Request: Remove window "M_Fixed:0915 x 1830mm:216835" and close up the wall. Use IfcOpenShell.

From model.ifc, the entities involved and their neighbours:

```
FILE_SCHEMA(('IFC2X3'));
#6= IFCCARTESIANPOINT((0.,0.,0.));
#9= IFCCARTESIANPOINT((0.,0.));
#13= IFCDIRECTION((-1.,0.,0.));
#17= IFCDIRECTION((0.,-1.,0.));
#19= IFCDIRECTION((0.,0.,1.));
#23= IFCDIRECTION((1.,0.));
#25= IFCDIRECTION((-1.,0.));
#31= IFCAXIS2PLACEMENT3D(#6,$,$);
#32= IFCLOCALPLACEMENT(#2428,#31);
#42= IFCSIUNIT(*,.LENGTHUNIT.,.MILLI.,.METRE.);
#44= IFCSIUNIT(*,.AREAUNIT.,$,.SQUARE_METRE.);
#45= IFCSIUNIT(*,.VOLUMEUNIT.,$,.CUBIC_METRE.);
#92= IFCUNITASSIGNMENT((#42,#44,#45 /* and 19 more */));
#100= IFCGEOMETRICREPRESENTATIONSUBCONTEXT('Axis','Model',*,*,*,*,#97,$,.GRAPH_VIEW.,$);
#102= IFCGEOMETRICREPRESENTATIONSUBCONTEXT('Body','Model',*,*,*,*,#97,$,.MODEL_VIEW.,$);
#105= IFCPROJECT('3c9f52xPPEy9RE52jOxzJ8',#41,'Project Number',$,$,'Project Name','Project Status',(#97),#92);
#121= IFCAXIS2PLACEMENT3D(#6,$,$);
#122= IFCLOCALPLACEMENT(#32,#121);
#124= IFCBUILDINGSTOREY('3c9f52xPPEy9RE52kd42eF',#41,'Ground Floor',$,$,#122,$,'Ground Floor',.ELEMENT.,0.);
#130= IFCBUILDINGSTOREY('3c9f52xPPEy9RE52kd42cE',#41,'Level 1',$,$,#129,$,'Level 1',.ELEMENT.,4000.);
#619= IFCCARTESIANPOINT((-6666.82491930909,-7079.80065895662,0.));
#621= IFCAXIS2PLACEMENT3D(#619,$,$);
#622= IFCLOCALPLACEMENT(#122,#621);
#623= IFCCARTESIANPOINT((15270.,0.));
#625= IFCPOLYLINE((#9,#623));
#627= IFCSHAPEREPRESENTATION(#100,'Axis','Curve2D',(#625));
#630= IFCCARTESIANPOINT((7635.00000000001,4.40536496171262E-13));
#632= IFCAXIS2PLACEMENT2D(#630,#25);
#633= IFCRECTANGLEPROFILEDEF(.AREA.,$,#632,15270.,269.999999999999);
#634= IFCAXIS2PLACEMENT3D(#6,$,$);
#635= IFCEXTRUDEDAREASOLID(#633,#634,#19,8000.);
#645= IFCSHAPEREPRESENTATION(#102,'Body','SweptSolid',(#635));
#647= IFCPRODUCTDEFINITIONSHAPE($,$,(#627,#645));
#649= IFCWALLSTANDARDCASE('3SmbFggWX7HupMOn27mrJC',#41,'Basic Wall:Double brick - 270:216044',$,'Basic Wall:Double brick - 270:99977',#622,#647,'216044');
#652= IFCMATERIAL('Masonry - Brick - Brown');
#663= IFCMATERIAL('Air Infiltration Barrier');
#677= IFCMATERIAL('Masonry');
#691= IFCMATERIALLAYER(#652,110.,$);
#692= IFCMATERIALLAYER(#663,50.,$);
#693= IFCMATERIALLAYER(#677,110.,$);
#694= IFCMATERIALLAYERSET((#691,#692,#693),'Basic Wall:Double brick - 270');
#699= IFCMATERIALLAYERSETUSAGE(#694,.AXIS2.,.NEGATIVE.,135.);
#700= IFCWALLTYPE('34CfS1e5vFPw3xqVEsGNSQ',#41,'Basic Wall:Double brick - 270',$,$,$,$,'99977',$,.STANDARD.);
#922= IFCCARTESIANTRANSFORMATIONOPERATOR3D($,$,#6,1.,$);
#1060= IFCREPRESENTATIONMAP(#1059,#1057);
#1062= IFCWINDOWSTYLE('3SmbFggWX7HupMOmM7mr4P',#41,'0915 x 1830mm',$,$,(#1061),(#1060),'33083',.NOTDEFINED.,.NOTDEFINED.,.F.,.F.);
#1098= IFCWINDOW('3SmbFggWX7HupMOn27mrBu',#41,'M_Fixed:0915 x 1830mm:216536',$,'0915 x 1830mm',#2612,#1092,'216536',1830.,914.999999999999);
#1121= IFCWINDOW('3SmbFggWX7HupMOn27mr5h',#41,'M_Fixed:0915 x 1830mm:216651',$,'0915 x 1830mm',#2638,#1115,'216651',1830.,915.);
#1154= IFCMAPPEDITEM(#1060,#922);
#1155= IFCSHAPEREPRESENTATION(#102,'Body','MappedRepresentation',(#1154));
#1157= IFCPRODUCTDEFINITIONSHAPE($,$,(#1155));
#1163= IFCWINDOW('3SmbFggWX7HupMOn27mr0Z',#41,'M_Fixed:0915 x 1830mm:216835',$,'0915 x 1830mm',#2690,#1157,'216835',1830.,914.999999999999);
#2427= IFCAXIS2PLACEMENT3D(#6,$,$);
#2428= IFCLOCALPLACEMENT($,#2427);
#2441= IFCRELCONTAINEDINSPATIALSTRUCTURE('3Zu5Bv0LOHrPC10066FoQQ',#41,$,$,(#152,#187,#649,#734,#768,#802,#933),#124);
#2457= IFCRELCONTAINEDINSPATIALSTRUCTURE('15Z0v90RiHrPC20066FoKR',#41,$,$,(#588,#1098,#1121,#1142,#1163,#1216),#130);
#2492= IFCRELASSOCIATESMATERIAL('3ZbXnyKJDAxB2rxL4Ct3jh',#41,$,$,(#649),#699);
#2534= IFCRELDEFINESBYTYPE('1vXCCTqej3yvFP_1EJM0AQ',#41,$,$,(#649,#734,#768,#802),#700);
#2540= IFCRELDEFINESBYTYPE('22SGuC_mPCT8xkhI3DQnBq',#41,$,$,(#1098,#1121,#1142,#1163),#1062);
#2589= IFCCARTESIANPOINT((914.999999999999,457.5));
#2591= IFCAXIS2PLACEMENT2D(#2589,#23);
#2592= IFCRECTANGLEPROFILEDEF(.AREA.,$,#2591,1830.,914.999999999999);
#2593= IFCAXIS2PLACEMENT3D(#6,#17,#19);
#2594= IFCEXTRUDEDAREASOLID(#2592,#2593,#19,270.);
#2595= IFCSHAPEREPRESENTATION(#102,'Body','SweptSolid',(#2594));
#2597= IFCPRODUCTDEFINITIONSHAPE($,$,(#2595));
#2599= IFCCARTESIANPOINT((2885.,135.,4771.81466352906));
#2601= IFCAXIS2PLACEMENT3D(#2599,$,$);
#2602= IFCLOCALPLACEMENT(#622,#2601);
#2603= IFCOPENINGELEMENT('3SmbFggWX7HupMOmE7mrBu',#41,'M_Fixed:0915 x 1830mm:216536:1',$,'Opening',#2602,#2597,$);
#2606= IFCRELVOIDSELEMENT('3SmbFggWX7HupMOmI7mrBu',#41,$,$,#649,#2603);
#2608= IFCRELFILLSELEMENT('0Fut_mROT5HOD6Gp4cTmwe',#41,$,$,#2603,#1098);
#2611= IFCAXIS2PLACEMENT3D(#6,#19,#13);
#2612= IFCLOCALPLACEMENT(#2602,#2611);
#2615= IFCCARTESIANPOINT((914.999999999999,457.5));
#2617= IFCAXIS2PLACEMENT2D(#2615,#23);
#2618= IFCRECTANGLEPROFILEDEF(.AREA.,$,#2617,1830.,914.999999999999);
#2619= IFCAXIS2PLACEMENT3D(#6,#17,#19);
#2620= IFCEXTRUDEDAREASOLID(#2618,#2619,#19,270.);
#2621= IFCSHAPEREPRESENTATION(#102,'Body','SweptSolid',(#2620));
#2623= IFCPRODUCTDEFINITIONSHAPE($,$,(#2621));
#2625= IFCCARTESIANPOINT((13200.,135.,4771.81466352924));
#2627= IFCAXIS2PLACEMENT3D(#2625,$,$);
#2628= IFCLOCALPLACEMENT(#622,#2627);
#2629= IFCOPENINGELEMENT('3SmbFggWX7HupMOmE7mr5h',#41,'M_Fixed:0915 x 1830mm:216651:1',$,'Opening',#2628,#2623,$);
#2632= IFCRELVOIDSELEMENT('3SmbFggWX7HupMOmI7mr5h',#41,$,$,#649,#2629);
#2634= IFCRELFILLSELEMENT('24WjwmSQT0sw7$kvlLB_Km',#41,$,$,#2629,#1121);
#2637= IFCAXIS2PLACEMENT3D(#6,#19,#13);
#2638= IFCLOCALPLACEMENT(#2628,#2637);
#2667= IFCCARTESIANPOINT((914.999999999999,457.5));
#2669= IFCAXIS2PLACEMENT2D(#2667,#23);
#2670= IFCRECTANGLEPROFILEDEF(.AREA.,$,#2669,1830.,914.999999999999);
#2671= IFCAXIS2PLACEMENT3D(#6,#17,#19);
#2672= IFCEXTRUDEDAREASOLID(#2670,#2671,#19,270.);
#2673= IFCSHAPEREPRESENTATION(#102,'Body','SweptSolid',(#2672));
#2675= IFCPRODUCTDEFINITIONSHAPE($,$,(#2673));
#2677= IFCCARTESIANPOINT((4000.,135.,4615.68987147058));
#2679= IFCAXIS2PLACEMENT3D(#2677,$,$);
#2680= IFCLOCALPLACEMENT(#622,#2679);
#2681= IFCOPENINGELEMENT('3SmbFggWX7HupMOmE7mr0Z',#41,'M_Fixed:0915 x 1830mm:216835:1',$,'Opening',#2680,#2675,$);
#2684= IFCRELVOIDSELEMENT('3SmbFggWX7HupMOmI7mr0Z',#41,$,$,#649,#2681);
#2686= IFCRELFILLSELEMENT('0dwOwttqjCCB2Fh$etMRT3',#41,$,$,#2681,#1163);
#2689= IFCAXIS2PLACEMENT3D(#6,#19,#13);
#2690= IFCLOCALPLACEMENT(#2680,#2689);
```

```python
import ifcopenshell
import ifcopenshell.api.feature
import ifcopenshell.api.root
import ifcopenshell.geom
import ifcopenshell.util.shape

model = ifcopenshell.open("model.ifc")
settings = ifcopenshell.geom.settings()


def volume(element):
    """Net volume in cubic metres, openings subtracted."""
    shape = ifcopenshell.geom.create_shape(settings, element)
    return ifcopenshell.util.shape.get_volume(shape.geometry)


window = model.by_id(1163)
opening = window.FillsVoids[0].RelatingOpeningElement
wall = opening.VoidsElements[0].RelatingBuildingElement
before = volume(wall)

ifcopenshell.api.root.remove_product(model, product=window)
ifcopenshell.api.feature.remove_feature(model, feature=opening)

after = volume(wall)

print(f"wall volume {before:.3f} -> {after:.3f} m3")

model.write("model_rev.ifc")
```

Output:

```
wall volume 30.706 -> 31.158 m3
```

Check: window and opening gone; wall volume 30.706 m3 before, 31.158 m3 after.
